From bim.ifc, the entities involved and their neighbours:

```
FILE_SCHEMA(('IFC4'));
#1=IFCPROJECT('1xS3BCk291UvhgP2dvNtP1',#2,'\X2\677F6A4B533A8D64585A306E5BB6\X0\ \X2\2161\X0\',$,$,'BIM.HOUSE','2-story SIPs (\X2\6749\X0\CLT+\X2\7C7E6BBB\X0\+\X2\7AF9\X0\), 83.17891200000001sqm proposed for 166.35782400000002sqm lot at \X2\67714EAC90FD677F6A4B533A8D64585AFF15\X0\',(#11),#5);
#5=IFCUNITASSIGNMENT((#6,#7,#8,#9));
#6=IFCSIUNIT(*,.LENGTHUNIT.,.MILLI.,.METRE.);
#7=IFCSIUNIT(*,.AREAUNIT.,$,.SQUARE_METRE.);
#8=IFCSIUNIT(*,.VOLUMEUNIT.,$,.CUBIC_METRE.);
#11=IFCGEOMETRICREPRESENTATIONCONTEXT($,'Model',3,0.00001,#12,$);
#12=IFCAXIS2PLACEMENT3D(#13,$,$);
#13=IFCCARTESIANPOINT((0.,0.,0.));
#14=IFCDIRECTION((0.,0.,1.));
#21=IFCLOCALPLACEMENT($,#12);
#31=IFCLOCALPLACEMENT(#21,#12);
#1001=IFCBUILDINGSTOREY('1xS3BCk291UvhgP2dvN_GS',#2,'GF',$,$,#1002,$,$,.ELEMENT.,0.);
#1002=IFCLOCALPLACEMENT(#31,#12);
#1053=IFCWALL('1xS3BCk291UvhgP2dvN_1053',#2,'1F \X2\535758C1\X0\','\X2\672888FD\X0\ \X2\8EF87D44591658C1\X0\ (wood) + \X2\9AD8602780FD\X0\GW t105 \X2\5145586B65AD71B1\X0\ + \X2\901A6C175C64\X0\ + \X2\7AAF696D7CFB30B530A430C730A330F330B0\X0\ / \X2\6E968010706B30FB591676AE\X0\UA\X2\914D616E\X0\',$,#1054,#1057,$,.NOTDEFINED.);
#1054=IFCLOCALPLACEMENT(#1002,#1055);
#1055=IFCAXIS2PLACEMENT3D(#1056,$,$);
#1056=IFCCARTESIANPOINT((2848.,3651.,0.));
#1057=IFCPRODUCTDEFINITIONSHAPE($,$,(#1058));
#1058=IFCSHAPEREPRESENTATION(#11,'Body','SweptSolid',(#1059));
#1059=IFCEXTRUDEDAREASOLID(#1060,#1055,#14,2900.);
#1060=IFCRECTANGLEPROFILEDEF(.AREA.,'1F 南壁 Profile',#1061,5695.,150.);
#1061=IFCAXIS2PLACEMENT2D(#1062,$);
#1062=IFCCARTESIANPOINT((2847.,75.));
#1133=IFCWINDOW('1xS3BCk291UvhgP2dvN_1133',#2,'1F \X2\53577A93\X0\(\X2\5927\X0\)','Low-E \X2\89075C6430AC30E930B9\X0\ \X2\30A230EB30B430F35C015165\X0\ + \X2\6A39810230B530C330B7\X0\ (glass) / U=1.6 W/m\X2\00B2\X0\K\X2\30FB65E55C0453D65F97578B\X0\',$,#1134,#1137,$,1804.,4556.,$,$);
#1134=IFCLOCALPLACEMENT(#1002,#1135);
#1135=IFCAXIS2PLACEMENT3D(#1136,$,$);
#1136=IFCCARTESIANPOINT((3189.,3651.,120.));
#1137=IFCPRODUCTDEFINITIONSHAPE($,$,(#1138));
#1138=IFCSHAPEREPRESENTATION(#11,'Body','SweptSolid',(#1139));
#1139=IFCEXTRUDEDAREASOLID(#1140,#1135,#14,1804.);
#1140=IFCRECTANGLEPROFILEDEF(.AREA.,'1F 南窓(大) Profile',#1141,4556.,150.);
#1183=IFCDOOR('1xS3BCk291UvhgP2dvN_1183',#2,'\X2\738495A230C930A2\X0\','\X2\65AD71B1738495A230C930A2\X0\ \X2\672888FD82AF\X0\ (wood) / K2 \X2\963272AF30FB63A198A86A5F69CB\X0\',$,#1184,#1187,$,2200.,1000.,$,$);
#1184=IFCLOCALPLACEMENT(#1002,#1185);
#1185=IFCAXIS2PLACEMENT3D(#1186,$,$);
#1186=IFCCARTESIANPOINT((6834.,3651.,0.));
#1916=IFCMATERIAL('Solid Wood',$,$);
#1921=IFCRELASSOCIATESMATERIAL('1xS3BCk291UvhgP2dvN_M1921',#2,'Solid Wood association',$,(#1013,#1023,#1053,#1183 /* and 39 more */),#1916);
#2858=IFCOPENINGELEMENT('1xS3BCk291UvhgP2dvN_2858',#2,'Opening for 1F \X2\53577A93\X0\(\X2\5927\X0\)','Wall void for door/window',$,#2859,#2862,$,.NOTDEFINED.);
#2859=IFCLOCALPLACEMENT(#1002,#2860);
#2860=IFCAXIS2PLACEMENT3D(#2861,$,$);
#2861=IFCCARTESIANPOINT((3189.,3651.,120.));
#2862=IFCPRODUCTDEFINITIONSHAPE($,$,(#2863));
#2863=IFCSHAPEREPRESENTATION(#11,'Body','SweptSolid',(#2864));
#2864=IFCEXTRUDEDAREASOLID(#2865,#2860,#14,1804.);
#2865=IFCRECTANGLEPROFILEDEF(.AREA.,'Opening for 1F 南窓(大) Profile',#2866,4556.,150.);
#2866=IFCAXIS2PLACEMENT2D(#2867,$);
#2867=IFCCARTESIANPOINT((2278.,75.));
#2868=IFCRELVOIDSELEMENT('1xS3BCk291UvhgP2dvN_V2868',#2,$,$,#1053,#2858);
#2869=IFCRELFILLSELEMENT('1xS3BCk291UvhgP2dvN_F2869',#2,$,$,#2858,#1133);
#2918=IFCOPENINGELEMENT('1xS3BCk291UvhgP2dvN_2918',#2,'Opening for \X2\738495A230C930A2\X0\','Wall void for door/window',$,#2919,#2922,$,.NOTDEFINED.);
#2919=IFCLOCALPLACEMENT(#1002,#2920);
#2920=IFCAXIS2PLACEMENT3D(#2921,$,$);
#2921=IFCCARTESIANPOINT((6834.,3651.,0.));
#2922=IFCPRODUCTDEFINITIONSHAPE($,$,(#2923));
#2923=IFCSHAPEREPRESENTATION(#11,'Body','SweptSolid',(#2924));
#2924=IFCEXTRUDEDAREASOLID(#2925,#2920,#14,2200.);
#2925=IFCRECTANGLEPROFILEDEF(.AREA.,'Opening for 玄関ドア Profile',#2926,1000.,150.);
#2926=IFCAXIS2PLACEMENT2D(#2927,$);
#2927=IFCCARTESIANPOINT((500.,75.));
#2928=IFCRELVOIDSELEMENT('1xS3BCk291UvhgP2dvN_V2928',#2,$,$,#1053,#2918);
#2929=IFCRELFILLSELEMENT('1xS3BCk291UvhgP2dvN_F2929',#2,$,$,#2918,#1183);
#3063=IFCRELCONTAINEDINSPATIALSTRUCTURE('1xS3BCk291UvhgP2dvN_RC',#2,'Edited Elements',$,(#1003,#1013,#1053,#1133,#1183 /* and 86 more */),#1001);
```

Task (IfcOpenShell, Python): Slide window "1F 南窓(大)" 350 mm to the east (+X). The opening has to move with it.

```python
import ifcopenshell
import ifcopenshell.api.geometry
import ifcopenshell.util.placement

model = ifcopenshell.open("bim.ifc")

window = model.by_guid("1xS3BCk291UvhgP2dvN_1133")
opening = window.FillsVoids[0].RelatingOpeningElement
wall = opening.VoidsElements[0].RelatingBuildingElement

wall_matrix = ifcopenshell.util.placement.get_local_placement(wall.ObjectPlacement)
shift = wall_matrix[:3, 0] * 350.0
before = ifcopenshell.util.placement.get_local_placement(window.ObjectPlacement)[:3, 3].copy()

# The window is not placed relative to its opening, so move both.
for product in (opening, window):
    matrix = ifcopenshell.util.placement.get_local_placement(product.ObjectPlacement)
    matrix[:3, 3] += shift
    ifcopenshell.api.geometry.edit_object_placement(model, product=product, matrix=matrix, is_si=False)

after = ifcopenshell.util.placement.get_local_placement(window.ObjectPlacement)[:3, 3]
print("window moved by", (after - before).round(3) + 0.0)

model.write("bim_v2.ifc")
```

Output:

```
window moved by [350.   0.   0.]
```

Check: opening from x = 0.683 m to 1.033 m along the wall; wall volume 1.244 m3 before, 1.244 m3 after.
